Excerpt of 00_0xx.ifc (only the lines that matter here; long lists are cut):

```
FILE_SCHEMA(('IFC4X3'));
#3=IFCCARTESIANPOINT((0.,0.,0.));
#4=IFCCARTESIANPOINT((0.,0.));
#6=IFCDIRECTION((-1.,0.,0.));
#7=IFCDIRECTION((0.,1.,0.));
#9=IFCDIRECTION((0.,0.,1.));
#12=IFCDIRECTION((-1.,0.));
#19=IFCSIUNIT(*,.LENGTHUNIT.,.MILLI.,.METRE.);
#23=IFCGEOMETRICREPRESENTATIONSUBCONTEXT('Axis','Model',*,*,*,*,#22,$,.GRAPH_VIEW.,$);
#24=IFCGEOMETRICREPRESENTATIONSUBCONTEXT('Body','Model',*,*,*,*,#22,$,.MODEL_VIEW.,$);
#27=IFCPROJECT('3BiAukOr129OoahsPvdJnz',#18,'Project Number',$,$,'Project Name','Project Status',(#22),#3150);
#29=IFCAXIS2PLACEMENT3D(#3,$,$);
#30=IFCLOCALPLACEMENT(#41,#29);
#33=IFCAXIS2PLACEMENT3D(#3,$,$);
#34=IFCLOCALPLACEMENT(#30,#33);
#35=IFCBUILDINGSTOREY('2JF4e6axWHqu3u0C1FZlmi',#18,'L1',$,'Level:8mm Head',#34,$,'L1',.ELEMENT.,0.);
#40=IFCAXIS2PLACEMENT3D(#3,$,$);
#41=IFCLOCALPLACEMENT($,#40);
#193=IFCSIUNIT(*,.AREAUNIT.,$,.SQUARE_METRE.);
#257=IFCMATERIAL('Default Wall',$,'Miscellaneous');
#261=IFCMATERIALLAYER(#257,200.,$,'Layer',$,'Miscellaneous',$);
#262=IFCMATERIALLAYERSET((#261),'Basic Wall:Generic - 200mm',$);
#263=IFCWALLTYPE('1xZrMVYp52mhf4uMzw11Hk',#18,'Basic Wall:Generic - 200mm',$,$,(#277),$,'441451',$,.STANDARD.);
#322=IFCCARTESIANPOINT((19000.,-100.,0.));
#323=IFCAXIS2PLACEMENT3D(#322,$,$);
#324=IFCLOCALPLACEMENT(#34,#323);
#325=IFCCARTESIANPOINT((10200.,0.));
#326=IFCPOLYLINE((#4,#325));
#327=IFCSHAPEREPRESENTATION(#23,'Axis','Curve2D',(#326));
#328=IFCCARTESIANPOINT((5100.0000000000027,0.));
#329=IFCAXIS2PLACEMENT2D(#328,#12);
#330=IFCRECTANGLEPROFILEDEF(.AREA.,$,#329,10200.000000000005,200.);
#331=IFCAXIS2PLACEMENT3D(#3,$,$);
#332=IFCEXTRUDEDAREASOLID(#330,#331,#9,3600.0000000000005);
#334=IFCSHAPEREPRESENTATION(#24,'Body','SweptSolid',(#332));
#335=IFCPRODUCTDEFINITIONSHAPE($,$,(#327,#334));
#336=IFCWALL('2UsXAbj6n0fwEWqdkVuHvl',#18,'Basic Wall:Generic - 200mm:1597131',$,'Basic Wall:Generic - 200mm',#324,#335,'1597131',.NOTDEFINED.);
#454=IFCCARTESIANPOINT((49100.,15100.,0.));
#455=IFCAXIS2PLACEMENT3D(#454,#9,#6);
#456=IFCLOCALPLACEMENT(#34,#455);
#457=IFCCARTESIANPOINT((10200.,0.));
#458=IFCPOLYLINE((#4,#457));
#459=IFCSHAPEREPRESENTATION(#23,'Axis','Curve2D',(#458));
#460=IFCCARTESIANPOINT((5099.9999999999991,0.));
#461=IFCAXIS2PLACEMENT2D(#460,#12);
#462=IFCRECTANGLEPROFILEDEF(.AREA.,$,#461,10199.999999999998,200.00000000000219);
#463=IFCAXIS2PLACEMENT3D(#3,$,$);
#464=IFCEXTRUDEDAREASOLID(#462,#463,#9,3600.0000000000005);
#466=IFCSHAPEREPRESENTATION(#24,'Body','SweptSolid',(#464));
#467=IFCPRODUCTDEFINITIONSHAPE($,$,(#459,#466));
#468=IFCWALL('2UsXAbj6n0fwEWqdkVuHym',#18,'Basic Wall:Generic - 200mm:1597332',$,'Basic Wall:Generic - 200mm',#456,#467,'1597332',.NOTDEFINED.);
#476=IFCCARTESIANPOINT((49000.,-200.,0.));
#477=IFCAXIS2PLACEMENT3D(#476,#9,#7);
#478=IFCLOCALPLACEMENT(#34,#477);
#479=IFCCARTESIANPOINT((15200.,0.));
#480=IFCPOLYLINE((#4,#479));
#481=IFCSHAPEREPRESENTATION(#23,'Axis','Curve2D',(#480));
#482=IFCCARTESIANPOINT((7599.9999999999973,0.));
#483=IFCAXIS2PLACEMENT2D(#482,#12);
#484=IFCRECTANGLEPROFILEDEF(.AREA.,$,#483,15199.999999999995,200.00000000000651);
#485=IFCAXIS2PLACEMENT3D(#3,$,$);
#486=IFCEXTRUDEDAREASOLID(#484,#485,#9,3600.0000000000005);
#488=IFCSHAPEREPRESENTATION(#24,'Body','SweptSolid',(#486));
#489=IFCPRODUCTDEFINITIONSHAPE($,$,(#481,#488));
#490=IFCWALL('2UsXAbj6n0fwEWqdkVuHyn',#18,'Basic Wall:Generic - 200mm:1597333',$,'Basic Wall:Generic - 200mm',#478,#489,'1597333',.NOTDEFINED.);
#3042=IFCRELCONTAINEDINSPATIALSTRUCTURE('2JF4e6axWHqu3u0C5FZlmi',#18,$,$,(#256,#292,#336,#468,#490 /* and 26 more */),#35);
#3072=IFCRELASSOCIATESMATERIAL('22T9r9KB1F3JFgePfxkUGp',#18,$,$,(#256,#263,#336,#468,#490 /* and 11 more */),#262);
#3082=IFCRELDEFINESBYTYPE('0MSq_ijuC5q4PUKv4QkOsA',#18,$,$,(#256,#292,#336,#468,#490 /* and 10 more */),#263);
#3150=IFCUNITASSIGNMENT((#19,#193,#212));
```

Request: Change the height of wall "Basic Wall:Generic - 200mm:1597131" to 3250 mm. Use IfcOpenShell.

```python
import ifcopenshell
import ifcopenshell.geom
import ifcopenshell.util.representation
import ifcopenshell.util.shape

model = ifcopenshell.open("00_0xx.ifc")
settings = ifcopenshell.geom.settings()


def volume(element):
    """Net volume in cubic metres, openings subtracted."""
    shape = ifcopenshell.geom.create_shape(settings, element)
    return ifcopenshell.util.shape.get_volume(shape.geometry)


wall = model.by_guid("2UsXAbj6n0fwEWqdkVuHvl")
before = volume(wall)

body = ifcopenshell.util.representation.get_representation(wall, "Model", "Body")
solid = body.Items[0]
old_height = solid.Depth
solid.Depth = 3250.0
after = volume(wall)

print(f"height {old_height:g} -> {solid.Depth:g}, volume {before:.3f} -> {after:.3f} m3")

model.write("00_0xx_rev.ifc")
```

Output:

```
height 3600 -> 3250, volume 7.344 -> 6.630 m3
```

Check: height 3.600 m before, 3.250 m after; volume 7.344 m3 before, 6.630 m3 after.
